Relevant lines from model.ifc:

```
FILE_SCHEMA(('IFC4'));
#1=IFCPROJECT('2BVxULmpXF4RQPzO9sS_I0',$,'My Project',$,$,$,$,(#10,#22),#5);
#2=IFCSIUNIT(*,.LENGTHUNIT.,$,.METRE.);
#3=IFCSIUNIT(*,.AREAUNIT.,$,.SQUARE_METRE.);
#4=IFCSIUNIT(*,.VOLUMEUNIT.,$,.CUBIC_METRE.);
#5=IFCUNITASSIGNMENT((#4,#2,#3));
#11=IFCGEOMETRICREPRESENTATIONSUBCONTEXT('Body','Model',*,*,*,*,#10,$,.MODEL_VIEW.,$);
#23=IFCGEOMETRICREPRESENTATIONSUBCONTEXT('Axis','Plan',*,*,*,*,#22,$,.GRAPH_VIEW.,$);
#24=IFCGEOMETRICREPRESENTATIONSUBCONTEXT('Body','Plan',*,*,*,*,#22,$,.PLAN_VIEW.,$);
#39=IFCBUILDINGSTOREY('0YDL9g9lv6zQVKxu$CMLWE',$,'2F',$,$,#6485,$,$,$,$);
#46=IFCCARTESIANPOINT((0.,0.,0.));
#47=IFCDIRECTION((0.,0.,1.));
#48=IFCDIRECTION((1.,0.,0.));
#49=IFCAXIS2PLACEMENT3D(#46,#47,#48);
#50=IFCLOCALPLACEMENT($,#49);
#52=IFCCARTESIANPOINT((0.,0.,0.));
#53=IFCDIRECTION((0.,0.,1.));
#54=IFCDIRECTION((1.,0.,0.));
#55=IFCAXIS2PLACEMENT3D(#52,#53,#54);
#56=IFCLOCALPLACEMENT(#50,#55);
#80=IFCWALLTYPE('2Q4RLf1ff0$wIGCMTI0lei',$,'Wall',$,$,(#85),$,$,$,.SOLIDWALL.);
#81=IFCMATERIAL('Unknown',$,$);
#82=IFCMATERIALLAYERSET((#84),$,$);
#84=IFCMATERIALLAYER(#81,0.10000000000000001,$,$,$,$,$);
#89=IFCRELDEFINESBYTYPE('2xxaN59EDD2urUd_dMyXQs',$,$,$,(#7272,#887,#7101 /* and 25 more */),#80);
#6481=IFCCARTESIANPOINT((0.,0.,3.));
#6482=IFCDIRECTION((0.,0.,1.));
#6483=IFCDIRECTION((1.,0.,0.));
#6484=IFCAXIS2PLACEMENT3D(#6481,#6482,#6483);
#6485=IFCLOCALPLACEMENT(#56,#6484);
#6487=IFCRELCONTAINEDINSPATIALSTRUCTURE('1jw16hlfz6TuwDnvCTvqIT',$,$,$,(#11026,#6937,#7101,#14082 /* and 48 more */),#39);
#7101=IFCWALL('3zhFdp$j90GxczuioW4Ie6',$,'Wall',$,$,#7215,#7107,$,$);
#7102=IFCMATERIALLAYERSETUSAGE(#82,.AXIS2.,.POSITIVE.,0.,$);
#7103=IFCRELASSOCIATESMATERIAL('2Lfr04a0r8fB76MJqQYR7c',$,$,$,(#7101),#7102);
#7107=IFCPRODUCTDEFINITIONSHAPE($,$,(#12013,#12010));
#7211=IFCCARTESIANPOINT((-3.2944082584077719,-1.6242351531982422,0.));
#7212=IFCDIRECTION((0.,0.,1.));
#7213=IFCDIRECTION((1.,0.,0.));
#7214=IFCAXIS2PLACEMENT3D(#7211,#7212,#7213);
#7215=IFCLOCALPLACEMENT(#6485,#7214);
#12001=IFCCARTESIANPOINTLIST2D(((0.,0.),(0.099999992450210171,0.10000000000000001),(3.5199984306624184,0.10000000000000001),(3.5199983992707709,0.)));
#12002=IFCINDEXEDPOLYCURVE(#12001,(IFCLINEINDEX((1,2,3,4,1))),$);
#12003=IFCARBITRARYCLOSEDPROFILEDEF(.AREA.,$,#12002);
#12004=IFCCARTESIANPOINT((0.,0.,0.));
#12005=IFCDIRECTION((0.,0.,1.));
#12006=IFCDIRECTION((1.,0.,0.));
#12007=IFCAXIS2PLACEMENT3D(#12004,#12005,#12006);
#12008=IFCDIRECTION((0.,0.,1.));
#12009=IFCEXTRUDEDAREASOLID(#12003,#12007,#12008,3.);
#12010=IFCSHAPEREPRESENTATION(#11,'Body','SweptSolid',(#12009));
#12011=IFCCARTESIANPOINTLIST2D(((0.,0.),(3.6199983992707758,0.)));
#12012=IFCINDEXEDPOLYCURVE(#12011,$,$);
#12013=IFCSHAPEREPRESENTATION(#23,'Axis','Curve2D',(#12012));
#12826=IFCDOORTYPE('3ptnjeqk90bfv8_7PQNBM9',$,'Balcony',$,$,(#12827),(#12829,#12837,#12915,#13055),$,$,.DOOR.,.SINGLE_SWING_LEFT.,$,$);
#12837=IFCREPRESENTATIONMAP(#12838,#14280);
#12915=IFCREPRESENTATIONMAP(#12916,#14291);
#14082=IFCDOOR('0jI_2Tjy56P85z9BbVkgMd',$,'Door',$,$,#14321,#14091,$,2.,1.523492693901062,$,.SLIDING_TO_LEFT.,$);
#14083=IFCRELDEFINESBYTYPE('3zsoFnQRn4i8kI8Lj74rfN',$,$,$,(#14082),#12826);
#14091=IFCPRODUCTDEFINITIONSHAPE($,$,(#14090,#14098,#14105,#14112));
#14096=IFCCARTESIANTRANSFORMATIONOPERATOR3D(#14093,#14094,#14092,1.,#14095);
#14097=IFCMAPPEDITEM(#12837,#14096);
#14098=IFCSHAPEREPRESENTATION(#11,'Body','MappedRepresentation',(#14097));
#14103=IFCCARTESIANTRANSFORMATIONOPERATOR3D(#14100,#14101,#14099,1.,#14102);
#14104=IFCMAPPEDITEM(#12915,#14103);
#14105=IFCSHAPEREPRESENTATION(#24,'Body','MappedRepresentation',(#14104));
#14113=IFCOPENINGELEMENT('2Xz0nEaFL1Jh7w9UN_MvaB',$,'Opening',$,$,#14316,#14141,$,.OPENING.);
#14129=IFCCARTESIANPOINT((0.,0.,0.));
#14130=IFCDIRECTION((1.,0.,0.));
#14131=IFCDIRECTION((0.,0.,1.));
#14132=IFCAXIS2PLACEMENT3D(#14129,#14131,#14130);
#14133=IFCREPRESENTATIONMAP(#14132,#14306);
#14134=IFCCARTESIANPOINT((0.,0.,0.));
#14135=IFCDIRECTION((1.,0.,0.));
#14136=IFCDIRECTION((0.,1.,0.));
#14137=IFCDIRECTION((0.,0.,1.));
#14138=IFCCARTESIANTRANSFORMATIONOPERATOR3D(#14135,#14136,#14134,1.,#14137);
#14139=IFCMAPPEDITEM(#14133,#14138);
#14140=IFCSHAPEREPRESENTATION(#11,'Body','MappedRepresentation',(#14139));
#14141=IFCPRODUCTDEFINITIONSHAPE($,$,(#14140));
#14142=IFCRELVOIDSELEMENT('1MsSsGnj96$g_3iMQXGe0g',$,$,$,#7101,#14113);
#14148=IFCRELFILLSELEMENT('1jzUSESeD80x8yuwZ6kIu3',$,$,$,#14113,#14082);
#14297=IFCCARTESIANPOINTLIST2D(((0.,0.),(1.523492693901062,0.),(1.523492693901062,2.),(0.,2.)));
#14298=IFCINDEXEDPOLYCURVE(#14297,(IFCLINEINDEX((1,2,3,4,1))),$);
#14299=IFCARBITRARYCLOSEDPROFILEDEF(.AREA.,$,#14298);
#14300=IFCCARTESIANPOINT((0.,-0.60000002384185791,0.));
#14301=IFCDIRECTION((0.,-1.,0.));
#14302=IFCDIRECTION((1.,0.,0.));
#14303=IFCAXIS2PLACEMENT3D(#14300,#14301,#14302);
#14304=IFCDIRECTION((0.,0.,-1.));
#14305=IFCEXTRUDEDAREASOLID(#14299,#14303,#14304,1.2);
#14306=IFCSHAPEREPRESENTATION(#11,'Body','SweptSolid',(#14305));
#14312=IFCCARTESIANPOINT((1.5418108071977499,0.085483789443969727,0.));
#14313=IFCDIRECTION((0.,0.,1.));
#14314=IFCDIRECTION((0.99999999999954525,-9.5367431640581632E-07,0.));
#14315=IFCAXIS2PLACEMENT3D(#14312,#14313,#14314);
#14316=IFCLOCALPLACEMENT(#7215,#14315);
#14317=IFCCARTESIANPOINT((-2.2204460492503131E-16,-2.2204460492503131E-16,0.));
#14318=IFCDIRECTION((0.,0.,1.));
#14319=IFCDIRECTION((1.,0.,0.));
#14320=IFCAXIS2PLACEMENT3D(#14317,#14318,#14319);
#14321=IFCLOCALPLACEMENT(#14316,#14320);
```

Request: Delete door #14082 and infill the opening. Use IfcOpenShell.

```python
import ifcopenshell
import ifcopenshell.api.feature
import ifcopenshell.api.root
import ifcopenshell.geom
import ifcopenshell.util.shape

model = ifcopenshell.open("model.ifc")
settings = ifcopenshell.geom.settings()


def volume(element):
    """Net volume in cubic metres, openings subtracted."""
    shape = ifcopenshell.geom.create_shape(settings, element)
    return ifcopenshell.util.shape.get_volume(shape.geometry)


door = model.by_guid("0jI_2Tjy56P85z9BbVkgMd")
opening = door.FillsVoids[0].RelatingOpeningElement
wall = opening.VoidsElements[0].RelatingBuildingElement
before = volume(wall)

ifcopenshell.api.root.remove_product(model, product=door)
ifcopenshell.api.feature.remove_feature(model, feature=opening)

after = volume(wall)

print(f"wall volume {before:.3f} -> {after:.3f} m3")

model.write("model_rev.ifc")
```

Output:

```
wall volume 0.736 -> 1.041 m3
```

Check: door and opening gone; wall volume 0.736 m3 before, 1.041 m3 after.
